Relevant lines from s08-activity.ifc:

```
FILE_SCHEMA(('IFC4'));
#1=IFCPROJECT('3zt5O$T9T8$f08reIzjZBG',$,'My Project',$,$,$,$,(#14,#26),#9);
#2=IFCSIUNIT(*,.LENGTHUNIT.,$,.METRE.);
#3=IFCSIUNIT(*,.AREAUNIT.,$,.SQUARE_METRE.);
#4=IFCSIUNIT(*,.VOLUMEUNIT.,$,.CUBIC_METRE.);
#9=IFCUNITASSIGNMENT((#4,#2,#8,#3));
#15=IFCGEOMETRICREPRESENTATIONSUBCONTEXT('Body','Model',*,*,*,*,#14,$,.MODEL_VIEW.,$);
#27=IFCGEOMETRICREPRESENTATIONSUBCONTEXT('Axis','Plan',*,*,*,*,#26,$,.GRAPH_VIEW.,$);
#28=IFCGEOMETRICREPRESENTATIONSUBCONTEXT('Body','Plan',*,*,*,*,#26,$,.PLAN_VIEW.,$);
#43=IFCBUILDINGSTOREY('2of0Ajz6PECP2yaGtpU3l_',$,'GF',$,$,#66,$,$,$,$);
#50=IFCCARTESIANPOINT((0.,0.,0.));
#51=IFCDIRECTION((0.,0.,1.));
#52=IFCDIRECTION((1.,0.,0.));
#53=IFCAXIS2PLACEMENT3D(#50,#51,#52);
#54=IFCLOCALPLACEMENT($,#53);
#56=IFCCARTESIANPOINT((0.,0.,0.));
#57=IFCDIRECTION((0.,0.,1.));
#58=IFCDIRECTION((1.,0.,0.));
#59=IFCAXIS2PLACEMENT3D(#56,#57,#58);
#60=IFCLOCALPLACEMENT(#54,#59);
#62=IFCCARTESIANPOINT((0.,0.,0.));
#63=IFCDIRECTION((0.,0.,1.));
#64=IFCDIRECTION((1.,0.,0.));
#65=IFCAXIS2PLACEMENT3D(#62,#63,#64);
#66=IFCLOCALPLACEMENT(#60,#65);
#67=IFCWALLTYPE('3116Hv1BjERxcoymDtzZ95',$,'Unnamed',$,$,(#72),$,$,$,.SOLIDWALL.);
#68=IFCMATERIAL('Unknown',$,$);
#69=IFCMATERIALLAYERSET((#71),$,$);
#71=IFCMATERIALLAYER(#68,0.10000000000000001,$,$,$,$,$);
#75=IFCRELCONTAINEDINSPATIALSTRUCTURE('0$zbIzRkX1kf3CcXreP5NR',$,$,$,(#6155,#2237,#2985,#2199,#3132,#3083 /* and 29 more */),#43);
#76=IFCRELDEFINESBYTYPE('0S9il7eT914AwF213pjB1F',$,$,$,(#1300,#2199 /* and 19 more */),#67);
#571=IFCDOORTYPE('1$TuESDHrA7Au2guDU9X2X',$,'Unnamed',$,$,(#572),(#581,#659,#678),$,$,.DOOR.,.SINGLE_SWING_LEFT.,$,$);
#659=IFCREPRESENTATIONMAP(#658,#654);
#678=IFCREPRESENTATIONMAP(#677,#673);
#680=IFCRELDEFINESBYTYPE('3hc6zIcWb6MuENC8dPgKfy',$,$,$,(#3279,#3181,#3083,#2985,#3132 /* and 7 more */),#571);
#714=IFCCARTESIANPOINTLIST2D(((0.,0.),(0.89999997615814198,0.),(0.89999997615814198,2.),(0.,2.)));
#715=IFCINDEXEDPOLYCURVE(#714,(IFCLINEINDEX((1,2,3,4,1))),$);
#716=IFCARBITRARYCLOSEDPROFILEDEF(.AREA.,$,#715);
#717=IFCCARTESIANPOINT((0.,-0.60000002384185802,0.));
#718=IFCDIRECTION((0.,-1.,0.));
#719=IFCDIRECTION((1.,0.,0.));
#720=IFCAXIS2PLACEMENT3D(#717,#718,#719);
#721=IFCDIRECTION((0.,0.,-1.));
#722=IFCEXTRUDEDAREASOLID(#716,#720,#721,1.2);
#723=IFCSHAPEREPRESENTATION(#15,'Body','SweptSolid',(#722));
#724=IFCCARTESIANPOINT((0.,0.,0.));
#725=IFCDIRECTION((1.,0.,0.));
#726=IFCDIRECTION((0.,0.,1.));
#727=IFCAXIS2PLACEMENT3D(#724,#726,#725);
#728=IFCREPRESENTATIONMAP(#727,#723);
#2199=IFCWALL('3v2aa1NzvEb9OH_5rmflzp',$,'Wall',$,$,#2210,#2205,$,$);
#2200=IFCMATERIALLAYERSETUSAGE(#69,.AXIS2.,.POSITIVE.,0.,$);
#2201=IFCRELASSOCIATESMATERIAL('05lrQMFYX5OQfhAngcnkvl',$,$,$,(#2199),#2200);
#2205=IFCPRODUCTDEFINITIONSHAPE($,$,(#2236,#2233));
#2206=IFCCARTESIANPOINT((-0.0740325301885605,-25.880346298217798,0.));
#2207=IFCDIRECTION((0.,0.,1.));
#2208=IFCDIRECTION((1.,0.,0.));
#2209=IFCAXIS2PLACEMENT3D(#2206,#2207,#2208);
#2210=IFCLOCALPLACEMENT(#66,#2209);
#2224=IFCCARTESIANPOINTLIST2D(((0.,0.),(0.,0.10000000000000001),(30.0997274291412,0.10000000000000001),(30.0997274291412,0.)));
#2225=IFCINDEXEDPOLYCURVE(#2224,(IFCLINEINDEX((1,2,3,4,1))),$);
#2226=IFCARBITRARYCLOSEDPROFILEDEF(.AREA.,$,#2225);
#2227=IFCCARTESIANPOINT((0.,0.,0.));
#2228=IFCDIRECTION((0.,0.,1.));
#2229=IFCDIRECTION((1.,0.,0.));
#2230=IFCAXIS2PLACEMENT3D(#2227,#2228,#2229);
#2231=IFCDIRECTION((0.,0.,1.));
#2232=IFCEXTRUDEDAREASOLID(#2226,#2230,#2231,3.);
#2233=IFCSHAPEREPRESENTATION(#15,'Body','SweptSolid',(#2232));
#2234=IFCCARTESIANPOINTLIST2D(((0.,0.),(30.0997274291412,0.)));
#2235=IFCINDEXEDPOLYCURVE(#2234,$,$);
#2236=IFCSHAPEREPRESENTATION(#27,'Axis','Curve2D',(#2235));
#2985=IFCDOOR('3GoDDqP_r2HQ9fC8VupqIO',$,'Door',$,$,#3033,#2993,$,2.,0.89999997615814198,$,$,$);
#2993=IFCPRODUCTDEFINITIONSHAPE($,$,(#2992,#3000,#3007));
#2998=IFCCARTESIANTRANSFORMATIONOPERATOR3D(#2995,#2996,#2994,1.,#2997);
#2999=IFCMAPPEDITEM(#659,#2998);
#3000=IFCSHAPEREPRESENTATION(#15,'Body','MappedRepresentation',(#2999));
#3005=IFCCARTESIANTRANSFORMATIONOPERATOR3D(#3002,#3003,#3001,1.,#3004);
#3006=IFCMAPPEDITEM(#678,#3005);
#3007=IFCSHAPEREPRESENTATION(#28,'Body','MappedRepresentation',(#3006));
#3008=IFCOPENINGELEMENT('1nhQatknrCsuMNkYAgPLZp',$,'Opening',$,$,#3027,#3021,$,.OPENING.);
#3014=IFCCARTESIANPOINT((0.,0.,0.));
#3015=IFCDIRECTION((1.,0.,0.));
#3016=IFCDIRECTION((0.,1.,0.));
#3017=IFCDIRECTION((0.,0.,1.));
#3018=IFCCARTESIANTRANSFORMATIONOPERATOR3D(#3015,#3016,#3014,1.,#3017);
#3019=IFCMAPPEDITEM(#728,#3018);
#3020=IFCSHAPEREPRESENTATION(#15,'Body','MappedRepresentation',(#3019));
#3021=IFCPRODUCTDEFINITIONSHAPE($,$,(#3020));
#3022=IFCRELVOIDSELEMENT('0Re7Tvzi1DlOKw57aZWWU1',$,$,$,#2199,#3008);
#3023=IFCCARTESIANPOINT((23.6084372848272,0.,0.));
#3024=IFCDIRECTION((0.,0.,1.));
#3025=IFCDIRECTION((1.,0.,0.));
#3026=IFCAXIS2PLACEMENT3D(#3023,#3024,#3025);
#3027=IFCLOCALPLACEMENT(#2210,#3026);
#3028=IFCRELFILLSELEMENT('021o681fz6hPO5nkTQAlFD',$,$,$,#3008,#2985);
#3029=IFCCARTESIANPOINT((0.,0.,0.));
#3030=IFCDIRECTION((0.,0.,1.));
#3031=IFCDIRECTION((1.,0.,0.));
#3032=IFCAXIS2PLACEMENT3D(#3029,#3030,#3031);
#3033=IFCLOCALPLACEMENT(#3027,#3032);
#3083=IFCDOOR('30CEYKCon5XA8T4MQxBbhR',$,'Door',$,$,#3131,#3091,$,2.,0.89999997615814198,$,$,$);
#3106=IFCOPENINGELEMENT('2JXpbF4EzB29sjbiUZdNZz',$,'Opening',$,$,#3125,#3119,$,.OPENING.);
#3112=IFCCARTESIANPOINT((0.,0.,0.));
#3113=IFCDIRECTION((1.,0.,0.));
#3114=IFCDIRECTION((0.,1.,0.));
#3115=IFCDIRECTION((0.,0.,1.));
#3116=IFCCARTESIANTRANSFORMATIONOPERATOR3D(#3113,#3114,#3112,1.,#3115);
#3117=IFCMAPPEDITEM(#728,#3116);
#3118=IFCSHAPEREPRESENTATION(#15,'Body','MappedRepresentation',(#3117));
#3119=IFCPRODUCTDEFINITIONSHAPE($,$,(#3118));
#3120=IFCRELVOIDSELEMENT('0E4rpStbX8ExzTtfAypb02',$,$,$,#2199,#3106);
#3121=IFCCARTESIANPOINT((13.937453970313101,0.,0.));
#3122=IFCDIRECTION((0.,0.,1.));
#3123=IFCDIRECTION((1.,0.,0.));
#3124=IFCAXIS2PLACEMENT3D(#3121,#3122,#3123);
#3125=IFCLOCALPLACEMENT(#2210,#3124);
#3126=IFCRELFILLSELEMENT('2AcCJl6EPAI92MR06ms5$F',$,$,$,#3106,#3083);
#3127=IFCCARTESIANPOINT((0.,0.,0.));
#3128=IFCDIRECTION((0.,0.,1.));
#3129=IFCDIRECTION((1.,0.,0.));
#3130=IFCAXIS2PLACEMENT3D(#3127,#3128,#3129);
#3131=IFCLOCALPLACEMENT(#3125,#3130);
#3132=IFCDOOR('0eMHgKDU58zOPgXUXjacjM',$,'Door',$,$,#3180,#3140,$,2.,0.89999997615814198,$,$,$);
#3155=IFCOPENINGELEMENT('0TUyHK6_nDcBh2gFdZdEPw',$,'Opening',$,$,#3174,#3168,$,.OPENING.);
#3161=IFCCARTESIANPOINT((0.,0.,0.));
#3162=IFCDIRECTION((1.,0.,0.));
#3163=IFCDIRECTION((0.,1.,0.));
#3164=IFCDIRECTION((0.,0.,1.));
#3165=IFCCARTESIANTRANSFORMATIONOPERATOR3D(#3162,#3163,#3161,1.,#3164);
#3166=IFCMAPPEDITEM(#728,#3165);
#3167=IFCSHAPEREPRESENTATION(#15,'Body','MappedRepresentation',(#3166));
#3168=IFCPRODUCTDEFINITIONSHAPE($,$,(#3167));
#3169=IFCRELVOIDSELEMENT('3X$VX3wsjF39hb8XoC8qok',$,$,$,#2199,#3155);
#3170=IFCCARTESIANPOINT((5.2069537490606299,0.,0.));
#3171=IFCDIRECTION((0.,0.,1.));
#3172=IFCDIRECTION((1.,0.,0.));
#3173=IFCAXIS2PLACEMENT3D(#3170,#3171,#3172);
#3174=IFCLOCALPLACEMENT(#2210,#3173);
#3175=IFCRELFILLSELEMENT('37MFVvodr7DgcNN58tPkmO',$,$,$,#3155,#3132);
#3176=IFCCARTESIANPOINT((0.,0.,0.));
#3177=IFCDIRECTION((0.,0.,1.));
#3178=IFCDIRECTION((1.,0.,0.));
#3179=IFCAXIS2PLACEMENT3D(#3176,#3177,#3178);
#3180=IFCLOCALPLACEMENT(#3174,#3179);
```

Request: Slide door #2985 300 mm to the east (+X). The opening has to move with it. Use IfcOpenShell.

```python
import ifcopenshell
import ifcopenshell.api.geometry
import ifcopenshell.util.placement

model = ifcopenshell.open("s08-activity.ifc")

door = model.by_guid("3GoDDqP_r2HQ9fC8VupqIO")
opening = door.FillsVoids[0].RelatingOpeningElement
wall = opening.VoidsElements[0].RelatingBuildingElement

wall_matrix = ifcopenshell.util.placement.get_local_placement(wall.ObjectPlacement)
shift = wall_matrix[:3, 0] * 0.3
before = ifcopenshell.util.placement.get_local_placement(door.ObjectPlacement)[:3, 3].copy()

# The door is placed relative to its opening, so it follows when the opening moves.
matrix = ifcopenshell.util.placement.get_local_placement(opening.ObjectPlacement)
matrix[:3, 3] += shift
ifcopenshell.api.geometry.edit_object_placement(
    model, product=opening, matrix=matrix, is_si=False, should_transform_children=True
)

after = ifcopenshell.util.placement.get_local_placement(door.ObjectPlacement)[:3, 3]
print("door moved by", (after - before).round(3) + 0.0)

model.write("s08-activity_rev.ifc")
```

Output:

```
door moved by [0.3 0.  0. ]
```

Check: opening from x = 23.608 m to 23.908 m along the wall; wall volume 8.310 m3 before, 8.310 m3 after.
